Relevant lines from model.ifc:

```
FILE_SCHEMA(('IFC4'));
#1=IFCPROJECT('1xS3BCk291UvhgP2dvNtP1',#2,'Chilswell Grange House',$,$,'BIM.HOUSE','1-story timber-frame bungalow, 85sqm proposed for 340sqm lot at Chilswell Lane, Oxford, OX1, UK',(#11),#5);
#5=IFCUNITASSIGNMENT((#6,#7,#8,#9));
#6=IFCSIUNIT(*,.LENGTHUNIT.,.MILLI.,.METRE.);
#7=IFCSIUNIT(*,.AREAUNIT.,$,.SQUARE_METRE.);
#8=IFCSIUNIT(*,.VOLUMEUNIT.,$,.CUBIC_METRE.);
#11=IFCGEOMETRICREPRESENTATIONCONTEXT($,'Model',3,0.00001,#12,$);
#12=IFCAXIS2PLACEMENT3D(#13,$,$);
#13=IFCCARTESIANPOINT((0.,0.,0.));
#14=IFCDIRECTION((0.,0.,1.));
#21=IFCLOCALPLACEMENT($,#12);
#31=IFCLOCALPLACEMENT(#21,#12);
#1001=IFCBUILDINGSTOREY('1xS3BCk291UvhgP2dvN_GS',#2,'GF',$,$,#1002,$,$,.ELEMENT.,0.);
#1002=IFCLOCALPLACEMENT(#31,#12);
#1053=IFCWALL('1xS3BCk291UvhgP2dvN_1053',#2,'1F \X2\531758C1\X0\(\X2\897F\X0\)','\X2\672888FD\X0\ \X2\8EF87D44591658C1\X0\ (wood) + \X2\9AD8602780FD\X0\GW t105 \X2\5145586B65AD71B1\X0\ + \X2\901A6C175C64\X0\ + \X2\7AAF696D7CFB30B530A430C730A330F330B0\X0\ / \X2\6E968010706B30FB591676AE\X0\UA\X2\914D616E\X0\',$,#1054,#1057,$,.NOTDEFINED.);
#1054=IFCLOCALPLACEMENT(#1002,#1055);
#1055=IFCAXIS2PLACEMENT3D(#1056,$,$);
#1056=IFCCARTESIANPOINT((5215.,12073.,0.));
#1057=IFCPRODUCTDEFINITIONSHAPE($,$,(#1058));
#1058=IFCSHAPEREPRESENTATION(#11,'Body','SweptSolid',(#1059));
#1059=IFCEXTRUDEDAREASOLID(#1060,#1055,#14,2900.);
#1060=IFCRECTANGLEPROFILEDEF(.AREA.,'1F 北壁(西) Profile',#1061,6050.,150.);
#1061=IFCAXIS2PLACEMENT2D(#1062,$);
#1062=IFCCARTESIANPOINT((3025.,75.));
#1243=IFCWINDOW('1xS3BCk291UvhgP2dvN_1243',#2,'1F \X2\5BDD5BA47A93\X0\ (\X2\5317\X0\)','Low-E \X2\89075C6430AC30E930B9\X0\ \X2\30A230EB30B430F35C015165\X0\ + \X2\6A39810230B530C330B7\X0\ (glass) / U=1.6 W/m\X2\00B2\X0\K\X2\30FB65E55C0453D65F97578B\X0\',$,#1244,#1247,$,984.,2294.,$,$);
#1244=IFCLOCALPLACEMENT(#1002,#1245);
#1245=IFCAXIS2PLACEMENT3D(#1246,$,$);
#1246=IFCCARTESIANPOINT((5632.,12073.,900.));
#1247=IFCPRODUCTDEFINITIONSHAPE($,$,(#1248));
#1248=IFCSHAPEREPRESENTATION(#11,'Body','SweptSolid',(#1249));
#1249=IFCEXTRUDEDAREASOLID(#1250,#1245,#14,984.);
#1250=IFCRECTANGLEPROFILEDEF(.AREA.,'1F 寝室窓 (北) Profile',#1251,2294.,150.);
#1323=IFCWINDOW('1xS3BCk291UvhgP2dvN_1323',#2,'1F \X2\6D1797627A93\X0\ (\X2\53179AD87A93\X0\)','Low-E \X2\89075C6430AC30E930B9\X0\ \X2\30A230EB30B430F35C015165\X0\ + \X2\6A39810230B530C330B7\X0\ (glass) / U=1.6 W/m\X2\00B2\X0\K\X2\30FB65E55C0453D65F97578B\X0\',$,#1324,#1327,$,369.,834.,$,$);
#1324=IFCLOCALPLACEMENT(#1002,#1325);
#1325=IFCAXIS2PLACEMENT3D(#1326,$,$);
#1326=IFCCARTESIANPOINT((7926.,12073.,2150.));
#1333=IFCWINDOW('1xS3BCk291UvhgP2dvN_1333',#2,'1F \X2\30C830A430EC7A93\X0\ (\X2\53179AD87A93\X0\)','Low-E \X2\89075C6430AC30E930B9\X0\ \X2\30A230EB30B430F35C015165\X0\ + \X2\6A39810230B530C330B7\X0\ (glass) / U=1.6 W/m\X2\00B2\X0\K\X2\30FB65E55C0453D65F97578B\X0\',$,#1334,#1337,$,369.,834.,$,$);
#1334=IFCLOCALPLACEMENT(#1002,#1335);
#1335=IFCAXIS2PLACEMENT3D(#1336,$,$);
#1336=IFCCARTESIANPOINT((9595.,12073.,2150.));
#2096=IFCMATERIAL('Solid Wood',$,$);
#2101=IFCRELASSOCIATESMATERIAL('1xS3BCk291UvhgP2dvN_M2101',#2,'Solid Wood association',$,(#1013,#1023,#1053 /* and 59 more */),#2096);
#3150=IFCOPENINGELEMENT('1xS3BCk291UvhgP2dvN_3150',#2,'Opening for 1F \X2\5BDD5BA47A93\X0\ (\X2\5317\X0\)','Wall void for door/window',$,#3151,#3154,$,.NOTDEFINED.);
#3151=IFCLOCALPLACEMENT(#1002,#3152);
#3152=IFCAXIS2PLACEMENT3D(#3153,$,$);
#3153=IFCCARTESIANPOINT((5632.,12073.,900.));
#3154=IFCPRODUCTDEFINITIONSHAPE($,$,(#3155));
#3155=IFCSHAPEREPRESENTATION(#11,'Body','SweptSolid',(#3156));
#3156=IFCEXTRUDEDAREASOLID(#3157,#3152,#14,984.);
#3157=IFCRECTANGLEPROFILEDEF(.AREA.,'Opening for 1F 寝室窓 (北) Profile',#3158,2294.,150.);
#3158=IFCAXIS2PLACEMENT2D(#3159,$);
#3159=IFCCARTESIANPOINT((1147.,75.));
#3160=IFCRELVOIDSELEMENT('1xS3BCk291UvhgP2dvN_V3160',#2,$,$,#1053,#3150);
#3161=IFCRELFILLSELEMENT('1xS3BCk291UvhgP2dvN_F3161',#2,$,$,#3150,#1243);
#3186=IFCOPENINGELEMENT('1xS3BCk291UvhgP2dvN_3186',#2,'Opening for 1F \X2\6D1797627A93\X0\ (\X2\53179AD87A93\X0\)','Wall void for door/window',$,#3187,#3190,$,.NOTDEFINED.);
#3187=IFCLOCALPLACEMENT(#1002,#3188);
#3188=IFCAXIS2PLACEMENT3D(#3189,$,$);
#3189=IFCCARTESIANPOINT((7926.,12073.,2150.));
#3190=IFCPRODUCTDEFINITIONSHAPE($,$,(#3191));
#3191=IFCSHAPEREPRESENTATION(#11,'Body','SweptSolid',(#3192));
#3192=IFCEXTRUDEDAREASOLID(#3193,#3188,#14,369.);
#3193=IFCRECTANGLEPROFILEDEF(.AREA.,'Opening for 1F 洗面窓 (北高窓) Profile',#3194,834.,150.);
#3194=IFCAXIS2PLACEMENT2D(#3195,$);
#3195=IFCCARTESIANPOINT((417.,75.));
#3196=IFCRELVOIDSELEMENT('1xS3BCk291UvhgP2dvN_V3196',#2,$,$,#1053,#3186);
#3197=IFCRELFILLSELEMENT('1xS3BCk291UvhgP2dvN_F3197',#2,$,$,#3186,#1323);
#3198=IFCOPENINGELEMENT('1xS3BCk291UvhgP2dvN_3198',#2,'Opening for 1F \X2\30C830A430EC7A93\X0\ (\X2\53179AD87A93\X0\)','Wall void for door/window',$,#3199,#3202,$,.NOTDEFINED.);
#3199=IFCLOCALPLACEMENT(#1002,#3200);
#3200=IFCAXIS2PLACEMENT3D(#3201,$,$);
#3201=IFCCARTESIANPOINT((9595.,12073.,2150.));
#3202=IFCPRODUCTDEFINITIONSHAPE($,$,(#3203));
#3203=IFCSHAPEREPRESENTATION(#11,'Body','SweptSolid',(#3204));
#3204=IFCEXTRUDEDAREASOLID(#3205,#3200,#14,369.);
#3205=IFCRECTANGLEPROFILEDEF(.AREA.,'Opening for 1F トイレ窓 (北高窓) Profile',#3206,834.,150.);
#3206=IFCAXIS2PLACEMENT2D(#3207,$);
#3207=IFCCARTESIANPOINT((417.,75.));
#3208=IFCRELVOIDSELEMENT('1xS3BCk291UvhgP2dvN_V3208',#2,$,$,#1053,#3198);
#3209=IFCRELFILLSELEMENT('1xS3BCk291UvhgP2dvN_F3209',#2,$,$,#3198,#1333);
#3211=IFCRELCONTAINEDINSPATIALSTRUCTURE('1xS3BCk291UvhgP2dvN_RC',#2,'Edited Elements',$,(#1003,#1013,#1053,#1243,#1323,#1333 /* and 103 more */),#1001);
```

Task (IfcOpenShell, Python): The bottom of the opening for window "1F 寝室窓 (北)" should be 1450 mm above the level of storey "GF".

```python
import numpy as np
import ifcopenshell
import ifcopenshell.api.geometry
import ifcopenshell.geom
import ifcopenshell.util.element
import ifcopenshell.util.placement
import ifcopenshell.util.shape
import ifcopenshell.util.unit

model = ifcopenshell.open("model.ifc")
unit_scale = ifcopenshell.util.unit.calculate_unit_scale(model)

window = model.by_guid("1xS3BCk291UvhgP2dvN_1243")
opening = window.FillsVoids[0].RelatingOpeningElement
storey = ifcopenshell.util.element.get_container(window, ifc_class="IfcBuildingStorey")
level = ifcopenshell.util.placement.get_local_placement(storey.ObjectPlacement)[2, 3]

# The opening's origin need not be at the sill, so measure its lowest point.
shape = ifcopenshell.geom.create_shape(ifcopenshell.geom.settings(), opening)
bottom = ifcopenshell.util.shape.get_shape_bottom_elevation(shape, shape.geometry) / unit_scale
dz = level + 1.45 / unit_scale - bottom

shift = np.array([0.0, 0.0, dz])
# The window is not placed relative to its opening, so move both.
for product in (opening, window):
    matrix = ifcopenshell.util.placement.get_local_placement(product.ObjectPlacement)
    matrix[:3, 3] += shift
    ifcopenshell.api.geometry.edit_object_placement(model, product=product, matrix=matrix, is_si=False)

print(f"moved by {dz * unit_scale:+.3f} m")

model.write("model_edited.ifc")
```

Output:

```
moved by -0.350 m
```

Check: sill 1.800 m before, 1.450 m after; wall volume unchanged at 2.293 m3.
